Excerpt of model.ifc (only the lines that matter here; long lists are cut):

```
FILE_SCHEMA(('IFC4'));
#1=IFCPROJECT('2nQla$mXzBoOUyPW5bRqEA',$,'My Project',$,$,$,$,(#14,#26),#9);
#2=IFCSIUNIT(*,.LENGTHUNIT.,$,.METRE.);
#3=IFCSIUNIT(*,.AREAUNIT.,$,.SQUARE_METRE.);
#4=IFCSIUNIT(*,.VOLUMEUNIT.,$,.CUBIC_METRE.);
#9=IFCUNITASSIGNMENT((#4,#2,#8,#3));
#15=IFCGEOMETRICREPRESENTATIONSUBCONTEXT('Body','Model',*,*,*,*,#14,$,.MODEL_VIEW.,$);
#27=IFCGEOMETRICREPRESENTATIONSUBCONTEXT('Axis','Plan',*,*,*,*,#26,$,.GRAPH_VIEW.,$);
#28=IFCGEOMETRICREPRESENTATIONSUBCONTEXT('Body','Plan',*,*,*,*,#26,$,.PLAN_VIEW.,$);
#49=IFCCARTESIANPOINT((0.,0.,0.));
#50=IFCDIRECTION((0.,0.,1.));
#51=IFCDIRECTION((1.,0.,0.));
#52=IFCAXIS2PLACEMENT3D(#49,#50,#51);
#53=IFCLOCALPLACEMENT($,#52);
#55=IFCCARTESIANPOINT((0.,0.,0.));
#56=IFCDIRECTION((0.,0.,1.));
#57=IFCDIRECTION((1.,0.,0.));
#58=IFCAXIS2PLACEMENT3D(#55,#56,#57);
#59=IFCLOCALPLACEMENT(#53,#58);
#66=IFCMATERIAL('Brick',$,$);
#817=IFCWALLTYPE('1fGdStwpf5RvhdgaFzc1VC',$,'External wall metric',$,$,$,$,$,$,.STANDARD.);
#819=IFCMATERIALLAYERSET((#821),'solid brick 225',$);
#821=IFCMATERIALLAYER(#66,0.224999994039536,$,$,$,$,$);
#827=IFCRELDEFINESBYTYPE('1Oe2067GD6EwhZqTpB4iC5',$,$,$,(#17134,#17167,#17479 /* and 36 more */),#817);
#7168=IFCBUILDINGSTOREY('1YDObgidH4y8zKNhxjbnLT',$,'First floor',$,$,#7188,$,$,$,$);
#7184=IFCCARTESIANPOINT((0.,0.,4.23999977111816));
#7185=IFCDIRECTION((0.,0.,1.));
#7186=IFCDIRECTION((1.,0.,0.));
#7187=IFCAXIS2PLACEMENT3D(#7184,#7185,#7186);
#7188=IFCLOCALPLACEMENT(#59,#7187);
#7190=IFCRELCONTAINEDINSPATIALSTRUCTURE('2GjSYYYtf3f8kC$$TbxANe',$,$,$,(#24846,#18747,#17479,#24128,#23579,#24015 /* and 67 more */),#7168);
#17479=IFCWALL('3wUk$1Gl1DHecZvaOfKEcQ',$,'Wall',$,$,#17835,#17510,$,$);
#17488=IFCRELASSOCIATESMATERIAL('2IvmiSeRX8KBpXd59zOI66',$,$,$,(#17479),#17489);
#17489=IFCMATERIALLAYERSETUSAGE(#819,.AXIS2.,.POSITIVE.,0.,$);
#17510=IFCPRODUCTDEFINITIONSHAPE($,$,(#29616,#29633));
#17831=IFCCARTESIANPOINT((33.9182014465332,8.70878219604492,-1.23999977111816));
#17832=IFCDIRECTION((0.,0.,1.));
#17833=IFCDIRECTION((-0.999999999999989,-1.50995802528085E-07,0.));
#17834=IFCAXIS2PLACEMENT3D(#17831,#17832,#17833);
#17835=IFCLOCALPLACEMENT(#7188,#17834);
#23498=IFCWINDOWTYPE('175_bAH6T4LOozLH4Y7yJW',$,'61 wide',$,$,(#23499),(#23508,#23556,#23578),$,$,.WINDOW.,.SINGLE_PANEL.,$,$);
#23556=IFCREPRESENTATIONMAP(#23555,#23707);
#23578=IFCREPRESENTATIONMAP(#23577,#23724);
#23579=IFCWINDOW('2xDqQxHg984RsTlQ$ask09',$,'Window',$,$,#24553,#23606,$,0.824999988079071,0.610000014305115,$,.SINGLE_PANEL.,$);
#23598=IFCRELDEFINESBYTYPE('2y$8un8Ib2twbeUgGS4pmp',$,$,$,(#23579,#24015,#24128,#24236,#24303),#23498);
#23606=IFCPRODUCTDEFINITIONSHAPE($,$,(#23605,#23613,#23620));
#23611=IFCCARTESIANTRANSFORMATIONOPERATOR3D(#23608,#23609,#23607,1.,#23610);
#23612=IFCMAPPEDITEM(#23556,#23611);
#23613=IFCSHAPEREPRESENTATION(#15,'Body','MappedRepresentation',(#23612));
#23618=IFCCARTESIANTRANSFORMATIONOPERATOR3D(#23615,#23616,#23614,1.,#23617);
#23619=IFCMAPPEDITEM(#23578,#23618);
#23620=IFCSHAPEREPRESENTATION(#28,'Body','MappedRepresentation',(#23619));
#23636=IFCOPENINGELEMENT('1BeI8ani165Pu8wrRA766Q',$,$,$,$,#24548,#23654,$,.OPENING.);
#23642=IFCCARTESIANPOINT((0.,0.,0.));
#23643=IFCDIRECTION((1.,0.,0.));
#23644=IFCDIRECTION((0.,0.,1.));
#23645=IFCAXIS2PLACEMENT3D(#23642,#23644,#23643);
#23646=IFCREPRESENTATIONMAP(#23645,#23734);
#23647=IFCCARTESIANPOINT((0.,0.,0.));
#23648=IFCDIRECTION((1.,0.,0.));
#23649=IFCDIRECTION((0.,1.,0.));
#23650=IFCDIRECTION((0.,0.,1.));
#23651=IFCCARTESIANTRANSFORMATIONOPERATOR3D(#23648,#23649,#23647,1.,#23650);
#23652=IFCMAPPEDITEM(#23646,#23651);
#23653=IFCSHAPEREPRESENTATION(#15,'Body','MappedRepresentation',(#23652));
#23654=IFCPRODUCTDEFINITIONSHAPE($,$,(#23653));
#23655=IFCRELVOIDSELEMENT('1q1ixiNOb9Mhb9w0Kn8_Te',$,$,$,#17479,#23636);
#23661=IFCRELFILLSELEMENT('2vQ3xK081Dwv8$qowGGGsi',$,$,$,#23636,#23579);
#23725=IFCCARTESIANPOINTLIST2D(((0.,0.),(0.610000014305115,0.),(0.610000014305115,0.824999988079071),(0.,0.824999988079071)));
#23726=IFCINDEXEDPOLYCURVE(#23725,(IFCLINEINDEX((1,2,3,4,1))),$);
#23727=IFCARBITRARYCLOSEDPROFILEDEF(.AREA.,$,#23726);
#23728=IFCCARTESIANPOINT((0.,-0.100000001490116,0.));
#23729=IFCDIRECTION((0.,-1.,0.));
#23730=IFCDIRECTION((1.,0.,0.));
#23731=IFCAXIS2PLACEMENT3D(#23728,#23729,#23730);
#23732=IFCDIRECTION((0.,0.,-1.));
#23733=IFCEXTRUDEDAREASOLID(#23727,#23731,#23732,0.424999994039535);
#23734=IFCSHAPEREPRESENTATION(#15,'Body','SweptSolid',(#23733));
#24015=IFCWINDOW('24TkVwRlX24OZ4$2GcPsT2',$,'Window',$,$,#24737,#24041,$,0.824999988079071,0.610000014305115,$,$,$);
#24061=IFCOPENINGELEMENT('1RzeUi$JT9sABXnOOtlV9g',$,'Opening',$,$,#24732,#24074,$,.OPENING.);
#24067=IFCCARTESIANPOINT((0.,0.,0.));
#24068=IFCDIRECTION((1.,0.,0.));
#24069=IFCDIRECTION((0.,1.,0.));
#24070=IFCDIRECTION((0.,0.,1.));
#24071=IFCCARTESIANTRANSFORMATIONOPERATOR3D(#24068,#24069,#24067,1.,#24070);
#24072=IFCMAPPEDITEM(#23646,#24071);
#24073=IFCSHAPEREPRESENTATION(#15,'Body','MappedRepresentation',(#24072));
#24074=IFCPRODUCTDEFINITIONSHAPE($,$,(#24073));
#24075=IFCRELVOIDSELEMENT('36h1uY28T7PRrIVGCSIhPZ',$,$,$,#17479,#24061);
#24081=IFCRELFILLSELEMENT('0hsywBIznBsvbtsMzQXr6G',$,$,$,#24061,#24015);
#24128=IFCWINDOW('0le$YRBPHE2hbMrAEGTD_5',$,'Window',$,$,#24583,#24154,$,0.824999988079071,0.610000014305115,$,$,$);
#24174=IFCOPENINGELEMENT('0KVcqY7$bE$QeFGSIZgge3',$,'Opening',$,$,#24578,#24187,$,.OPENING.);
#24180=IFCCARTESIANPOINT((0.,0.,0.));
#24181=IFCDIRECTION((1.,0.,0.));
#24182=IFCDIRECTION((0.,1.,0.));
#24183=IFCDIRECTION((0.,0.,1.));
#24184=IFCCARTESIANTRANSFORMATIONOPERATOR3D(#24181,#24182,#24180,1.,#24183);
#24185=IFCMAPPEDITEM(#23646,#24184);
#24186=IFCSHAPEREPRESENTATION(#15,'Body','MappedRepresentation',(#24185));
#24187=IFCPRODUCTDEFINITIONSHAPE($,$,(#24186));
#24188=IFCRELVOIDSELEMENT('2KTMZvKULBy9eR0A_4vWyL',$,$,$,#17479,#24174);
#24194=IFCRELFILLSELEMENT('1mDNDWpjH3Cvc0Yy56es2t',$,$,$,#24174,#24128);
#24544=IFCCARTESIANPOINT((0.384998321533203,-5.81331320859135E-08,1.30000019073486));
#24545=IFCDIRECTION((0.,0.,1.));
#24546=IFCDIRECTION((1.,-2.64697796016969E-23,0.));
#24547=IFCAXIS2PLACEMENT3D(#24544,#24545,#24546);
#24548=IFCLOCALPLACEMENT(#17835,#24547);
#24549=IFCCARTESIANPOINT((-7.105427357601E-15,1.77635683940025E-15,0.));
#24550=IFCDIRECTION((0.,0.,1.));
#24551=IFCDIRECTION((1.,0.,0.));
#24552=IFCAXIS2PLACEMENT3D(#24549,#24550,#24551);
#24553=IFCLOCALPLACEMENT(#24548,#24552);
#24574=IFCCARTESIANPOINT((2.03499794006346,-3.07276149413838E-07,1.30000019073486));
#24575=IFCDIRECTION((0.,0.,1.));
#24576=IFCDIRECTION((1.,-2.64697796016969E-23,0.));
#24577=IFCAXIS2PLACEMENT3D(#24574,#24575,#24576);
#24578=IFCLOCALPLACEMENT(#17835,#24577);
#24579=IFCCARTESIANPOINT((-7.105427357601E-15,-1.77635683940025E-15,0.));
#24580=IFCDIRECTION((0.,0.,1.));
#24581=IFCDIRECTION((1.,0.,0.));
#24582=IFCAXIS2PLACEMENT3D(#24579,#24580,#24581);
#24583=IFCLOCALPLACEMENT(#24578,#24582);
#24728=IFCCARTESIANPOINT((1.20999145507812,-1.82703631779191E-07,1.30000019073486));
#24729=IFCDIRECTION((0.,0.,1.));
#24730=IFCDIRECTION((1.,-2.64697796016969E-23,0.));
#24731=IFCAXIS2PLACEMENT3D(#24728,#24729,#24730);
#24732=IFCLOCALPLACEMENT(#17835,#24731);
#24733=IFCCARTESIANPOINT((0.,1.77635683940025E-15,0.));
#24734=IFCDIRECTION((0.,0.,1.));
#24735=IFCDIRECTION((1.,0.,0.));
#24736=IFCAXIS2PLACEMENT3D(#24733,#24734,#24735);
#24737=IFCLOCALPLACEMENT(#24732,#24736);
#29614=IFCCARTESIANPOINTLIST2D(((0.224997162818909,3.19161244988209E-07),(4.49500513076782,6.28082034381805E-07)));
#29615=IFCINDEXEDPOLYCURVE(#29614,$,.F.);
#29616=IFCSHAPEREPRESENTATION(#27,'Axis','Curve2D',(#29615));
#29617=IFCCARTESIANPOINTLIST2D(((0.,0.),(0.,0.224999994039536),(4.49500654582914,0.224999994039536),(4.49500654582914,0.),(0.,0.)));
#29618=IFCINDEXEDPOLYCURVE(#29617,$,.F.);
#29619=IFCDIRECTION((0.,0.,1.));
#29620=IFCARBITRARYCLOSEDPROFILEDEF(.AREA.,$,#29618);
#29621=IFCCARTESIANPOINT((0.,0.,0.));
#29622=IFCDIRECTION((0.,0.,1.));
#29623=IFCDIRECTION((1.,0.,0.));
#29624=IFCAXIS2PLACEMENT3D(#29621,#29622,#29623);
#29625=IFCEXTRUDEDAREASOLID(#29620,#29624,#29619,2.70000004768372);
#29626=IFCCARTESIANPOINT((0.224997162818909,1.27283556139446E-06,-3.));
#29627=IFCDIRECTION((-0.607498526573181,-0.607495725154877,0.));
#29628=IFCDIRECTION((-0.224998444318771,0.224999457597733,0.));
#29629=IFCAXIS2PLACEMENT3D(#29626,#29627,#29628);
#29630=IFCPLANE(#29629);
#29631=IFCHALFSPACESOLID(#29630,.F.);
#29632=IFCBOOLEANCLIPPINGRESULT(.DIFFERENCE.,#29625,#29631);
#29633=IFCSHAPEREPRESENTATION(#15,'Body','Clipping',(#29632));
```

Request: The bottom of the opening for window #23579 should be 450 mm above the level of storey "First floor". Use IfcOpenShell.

```python
import numpy as np
import ifcopenshell
import ifcopenshell.api.geometry
import ifcopenshell.geom
import ifcopenshell.util.element
import ifcopenshell.util.placement
import ifcopenshell.util.shape
import ifcopenshell.util.unit

model = ifcopenshell.open("model.ifc")
unit_scale = ifcopenshell.util.unit.calculate_unit_scale(model)

window = model.by_guid("2xDqQxHg984RsTlQ$ask09")
opening = window.FillsVoids[0].RelatingOpeningElement
storey = ifcopenshell.util.element.get_container(window, ifc_class="IfcBuildingStorey")
level = ifcopenshell.util.placement.get_local_placement(storey.ObjectPlacement)[2, 3]

# The opening's origin need not be at the sill, so measure its lowest point.
shape = ifcopenshell.geom.create_shape(ifcopenshell.geom.settings(), opening)
bottom = ifcopenshell.util.shape.get_shape_bottom_elevation(shape, shape.geometry) / unit_scale
dz = level + 0.45 / unit_scale - bottom

shift = np.array([0.0, 0.0, dz])
# The window is placed relative to its opening, so it follows when the opening moves.
matrix = ifcopenshell.util.placement.get_local_placement(opening.ObjectPlacement)
matrix[:3, 3] += shift
ifcopenshell.api.geometry.edit_object_placement(
    model, product=opening, matrix=matrix, is_si=False, should_transform_children=True
)

print(f"moved by {dz * unit_scale:+.3f} m")

model.write("model_v2.ifc")
```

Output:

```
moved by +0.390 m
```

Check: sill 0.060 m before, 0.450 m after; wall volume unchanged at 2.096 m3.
